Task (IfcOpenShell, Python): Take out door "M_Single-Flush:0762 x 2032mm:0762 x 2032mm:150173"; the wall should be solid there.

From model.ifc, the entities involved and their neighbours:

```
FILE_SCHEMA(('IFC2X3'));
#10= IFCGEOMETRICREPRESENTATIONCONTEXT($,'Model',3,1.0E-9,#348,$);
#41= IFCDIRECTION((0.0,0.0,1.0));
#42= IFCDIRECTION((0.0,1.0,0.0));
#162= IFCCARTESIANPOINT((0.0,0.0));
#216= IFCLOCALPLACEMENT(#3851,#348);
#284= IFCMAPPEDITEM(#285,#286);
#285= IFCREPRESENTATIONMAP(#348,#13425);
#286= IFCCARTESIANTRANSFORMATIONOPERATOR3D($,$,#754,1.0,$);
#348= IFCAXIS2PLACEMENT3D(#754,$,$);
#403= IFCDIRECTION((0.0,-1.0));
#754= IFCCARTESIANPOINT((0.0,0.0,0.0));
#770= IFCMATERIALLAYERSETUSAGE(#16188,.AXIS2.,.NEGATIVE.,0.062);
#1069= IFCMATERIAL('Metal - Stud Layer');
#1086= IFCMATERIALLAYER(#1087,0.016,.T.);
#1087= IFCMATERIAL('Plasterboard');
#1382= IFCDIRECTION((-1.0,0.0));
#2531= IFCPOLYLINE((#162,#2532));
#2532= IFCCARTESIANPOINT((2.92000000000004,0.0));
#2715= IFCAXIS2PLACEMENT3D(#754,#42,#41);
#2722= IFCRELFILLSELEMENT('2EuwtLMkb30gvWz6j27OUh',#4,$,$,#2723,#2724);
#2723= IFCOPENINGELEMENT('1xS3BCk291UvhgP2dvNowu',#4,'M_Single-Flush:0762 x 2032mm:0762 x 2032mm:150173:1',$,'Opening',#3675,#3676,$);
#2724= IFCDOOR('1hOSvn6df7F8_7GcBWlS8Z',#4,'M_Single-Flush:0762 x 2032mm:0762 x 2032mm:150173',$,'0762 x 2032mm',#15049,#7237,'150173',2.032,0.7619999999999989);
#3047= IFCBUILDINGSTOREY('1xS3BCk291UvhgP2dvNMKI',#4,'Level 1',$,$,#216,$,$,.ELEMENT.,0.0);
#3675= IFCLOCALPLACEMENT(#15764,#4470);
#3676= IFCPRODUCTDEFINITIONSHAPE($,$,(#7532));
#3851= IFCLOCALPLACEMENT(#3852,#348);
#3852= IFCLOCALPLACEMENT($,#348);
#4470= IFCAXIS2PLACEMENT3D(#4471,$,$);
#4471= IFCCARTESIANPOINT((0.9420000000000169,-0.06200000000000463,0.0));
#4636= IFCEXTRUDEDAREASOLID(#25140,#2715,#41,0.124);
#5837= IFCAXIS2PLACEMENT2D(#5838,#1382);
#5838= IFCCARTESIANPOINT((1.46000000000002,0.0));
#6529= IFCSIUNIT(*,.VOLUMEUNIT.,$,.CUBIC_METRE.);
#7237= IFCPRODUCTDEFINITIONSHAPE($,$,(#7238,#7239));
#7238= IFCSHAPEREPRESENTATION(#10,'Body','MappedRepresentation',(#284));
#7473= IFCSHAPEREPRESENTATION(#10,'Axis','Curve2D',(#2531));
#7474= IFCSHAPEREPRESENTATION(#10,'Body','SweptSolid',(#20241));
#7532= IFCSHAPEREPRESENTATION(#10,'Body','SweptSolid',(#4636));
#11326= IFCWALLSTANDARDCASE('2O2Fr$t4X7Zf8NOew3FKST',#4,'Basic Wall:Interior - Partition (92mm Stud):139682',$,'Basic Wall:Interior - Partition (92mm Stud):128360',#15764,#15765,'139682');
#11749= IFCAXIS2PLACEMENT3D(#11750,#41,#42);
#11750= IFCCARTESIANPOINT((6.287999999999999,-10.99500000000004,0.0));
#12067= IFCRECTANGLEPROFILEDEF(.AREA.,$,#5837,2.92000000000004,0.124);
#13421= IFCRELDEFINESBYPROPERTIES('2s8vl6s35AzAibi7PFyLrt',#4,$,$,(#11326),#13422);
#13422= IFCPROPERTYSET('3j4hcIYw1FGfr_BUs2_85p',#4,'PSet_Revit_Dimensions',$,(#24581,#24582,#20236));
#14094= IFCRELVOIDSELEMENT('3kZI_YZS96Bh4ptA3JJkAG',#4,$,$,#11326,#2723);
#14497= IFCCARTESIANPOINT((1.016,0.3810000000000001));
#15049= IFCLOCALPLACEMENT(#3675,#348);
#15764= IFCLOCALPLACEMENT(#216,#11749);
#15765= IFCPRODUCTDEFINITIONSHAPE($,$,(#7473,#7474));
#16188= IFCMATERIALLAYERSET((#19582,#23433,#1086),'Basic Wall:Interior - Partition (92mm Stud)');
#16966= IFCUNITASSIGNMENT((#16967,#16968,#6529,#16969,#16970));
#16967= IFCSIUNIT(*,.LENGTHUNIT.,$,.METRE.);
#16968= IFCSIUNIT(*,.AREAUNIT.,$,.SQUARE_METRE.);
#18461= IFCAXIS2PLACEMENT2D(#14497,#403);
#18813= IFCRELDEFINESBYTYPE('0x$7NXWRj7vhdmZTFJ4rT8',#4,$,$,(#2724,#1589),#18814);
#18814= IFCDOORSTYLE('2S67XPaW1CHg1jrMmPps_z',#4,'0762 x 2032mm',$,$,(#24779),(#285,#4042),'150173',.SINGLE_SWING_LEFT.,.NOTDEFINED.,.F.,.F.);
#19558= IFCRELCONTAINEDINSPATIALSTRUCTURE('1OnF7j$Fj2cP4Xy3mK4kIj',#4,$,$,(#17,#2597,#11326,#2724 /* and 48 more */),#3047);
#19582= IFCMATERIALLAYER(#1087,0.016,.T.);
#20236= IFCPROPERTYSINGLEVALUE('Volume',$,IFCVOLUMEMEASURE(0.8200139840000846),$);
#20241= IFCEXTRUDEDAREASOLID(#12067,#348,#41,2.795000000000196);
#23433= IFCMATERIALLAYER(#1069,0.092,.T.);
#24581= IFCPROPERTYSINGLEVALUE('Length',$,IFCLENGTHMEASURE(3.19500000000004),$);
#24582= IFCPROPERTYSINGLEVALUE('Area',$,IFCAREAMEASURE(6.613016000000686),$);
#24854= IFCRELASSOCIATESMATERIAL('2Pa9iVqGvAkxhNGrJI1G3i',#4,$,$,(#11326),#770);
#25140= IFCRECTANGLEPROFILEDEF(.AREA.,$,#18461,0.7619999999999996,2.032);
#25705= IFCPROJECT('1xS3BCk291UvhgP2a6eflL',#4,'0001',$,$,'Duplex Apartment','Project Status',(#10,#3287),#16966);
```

```python
import ifcopenshell
import ifcopenshell.api.feature
import ifcopenshell.api.pset
import ifcopenshell.api.root
import ifcopenshell.geom
import ifcopenshell.util.element
import ifcopenshell.util.shape
import ifcopenshell.util.unit

model = ifcopenshell.open("model.ifc")
area_scale = ifcopenshell.util.unit.calculate_unit_scale(model, "AREAUNIT")
volume_scale = ifcopenshell.util.unit.calculate_unit_scale(model, "VOLUMEUNIT")
settings = ifcopenshell.geom.settings()


def volume(element):
    """Net volume in cubic metres, openings subtracted."""
    shape = ifcopenshell.geom.create_shape(settings, element)
    return ifcopenshell.util.shape.get_volume(shape.geometry)


door = model.by_id(2724)
opening = door.FillsVoids[0].RelatingOpeningElement
wall = opening.VoidsElements[0].RelatingBuildingElement
before = volume(wall)

ifcopenshell.api.root.remove_product(model, product=door)
ifcopenshell.api.feature.remove_feature(model, feature=opening)

after = volume(wall)
thickness = 0.124  # wall thickness in metres

# Update the wall's stored quantities.
pset = model.by_id(ifcopenshell.util.element.get_pset(wall, "PSet_Revit_Dimensions", should_inherit=False)["id"])
ifcopenshell.api.pset.edit_pset(model, pset=pset, properties={
    "Area": model.create_entity("IfcAreaMeasure", after / thickness / area_scale),
    "Volume": model.create_entity("IfcVolumeMeasure", after / volume_scale),
})

print(f"wall volume {before:.3f} -> {after:.3f} m3")

model.write("model_edited.ifc")
```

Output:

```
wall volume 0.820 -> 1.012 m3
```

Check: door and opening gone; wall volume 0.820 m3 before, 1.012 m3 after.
